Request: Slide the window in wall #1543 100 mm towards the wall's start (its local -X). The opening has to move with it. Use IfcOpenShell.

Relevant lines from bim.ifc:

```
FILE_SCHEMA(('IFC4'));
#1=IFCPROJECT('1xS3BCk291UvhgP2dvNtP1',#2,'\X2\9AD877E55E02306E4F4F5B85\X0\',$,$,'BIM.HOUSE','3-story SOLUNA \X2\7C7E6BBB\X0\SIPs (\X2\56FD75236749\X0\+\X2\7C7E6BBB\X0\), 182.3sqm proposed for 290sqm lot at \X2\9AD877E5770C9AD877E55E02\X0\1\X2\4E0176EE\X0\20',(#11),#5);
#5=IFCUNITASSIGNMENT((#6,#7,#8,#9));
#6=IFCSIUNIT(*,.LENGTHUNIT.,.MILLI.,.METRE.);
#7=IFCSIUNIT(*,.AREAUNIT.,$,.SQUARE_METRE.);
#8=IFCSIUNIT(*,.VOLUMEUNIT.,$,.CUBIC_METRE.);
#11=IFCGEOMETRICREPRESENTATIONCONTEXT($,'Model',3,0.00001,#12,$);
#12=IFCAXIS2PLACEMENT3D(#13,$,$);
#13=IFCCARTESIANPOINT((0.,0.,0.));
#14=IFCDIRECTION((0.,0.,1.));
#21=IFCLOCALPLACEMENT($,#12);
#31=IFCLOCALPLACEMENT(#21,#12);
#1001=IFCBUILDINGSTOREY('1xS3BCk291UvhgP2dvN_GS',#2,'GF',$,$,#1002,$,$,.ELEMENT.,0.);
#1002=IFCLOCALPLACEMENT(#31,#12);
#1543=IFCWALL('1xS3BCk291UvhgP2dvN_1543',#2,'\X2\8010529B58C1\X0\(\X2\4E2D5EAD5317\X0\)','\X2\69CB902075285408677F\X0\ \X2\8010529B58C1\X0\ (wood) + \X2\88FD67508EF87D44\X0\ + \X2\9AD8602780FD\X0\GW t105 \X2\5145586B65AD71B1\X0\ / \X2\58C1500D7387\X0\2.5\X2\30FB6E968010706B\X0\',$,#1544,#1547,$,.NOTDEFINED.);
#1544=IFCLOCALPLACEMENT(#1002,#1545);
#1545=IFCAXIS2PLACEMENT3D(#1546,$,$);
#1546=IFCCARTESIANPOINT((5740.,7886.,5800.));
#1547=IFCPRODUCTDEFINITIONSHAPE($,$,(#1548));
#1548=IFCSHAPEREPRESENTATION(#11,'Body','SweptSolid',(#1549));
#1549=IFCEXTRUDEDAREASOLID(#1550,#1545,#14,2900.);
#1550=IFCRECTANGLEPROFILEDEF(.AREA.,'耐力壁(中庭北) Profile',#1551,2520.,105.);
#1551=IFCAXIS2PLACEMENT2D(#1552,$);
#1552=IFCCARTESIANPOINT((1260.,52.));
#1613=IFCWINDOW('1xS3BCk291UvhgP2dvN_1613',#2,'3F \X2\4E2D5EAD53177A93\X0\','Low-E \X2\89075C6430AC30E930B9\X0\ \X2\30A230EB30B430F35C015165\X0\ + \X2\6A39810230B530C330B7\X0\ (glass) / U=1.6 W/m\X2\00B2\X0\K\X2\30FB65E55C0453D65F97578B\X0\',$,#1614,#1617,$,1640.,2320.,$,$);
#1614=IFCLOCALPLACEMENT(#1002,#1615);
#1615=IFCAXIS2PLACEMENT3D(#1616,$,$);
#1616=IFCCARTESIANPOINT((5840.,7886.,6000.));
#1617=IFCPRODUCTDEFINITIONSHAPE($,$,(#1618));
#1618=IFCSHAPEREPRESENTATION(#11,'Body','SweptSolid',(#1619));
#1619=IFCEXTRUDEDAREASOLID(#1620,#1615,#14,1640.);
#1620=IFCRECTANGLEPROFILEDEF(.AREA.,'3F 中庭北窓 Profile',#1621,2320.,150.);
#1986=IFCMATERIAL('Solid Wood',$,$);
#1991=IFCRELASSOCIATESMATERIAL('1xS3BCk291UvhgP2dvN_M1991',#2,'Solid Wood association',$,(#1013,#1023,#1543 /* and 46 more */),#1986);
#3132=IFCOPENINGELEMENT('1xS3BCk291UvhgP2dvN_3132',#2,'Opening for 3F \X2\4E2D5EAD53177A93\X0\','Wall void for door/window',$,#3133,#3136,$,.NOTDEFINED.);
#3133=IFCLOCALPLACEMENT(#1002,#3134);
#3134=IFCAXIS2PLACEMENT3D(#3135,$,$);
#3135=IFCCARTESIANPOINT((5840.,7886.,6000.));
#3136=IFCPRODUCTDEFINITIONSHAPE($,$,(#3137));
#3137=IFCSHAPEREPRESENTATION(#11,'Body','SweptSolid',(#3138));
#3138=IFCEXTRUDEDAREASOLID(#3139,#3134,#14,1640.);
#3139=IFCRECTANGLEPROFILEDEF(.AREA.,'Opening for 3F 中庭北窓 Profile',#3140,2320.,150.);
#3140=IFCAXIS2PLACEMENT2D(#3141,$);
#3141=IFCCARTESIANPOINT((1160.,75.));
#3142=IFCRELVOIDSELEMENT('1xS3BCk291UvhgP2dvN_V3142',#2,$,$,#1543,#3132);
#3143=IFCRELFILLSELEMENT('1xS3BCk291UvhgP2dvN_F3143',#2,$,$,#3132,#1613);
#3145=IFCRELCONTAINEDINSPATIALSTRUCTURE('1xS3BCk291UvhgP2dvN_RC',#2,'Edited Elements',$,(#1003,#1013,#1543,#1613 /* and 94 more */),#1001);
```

```python
import ifcopenshell
import ifcopenshell.api.geometry
import ifcopenshell.util.placement

model = ifcopenshell.open("bim.ifc")

window = model.by_id(1613)
opening = window.FillsVoids[0].RelatingOpeningElement
wall = opening.VoidsElements[0].RelatingBuildingElement

wall_matrix = ifcopenshell.util.placement.get_local_placement(wall.ObjectPlacement)
shift = wall_matrix[:3, 0] * -100.0
before = ifcopenshell.util.placement.get_local_placement(window.ObjectPlacement)[:3, 3].copy()

# The window is not placed relative to its opening, so move both.
for product in (opening, window):
    matrix = ifcopenshell.util.placement.get_local_placement(product.ObjectPlacement)
    matrix[:3, 3] += shift
    ifcopenshell.api.geometry.edit_object_placement(model, product=product, matrix=matrix, is_si=False)

after = ifcopenshell.util.placement.get_local_placement(window.ObjectPlacement)[:3, 3]
print("window moved by", (after - before).round(3) + 0.0)

model.write("bim_v2.ifc")
```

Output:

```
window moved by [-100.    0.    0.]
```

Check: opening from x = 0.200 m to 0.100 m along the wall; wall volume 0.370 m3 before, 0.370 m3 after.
